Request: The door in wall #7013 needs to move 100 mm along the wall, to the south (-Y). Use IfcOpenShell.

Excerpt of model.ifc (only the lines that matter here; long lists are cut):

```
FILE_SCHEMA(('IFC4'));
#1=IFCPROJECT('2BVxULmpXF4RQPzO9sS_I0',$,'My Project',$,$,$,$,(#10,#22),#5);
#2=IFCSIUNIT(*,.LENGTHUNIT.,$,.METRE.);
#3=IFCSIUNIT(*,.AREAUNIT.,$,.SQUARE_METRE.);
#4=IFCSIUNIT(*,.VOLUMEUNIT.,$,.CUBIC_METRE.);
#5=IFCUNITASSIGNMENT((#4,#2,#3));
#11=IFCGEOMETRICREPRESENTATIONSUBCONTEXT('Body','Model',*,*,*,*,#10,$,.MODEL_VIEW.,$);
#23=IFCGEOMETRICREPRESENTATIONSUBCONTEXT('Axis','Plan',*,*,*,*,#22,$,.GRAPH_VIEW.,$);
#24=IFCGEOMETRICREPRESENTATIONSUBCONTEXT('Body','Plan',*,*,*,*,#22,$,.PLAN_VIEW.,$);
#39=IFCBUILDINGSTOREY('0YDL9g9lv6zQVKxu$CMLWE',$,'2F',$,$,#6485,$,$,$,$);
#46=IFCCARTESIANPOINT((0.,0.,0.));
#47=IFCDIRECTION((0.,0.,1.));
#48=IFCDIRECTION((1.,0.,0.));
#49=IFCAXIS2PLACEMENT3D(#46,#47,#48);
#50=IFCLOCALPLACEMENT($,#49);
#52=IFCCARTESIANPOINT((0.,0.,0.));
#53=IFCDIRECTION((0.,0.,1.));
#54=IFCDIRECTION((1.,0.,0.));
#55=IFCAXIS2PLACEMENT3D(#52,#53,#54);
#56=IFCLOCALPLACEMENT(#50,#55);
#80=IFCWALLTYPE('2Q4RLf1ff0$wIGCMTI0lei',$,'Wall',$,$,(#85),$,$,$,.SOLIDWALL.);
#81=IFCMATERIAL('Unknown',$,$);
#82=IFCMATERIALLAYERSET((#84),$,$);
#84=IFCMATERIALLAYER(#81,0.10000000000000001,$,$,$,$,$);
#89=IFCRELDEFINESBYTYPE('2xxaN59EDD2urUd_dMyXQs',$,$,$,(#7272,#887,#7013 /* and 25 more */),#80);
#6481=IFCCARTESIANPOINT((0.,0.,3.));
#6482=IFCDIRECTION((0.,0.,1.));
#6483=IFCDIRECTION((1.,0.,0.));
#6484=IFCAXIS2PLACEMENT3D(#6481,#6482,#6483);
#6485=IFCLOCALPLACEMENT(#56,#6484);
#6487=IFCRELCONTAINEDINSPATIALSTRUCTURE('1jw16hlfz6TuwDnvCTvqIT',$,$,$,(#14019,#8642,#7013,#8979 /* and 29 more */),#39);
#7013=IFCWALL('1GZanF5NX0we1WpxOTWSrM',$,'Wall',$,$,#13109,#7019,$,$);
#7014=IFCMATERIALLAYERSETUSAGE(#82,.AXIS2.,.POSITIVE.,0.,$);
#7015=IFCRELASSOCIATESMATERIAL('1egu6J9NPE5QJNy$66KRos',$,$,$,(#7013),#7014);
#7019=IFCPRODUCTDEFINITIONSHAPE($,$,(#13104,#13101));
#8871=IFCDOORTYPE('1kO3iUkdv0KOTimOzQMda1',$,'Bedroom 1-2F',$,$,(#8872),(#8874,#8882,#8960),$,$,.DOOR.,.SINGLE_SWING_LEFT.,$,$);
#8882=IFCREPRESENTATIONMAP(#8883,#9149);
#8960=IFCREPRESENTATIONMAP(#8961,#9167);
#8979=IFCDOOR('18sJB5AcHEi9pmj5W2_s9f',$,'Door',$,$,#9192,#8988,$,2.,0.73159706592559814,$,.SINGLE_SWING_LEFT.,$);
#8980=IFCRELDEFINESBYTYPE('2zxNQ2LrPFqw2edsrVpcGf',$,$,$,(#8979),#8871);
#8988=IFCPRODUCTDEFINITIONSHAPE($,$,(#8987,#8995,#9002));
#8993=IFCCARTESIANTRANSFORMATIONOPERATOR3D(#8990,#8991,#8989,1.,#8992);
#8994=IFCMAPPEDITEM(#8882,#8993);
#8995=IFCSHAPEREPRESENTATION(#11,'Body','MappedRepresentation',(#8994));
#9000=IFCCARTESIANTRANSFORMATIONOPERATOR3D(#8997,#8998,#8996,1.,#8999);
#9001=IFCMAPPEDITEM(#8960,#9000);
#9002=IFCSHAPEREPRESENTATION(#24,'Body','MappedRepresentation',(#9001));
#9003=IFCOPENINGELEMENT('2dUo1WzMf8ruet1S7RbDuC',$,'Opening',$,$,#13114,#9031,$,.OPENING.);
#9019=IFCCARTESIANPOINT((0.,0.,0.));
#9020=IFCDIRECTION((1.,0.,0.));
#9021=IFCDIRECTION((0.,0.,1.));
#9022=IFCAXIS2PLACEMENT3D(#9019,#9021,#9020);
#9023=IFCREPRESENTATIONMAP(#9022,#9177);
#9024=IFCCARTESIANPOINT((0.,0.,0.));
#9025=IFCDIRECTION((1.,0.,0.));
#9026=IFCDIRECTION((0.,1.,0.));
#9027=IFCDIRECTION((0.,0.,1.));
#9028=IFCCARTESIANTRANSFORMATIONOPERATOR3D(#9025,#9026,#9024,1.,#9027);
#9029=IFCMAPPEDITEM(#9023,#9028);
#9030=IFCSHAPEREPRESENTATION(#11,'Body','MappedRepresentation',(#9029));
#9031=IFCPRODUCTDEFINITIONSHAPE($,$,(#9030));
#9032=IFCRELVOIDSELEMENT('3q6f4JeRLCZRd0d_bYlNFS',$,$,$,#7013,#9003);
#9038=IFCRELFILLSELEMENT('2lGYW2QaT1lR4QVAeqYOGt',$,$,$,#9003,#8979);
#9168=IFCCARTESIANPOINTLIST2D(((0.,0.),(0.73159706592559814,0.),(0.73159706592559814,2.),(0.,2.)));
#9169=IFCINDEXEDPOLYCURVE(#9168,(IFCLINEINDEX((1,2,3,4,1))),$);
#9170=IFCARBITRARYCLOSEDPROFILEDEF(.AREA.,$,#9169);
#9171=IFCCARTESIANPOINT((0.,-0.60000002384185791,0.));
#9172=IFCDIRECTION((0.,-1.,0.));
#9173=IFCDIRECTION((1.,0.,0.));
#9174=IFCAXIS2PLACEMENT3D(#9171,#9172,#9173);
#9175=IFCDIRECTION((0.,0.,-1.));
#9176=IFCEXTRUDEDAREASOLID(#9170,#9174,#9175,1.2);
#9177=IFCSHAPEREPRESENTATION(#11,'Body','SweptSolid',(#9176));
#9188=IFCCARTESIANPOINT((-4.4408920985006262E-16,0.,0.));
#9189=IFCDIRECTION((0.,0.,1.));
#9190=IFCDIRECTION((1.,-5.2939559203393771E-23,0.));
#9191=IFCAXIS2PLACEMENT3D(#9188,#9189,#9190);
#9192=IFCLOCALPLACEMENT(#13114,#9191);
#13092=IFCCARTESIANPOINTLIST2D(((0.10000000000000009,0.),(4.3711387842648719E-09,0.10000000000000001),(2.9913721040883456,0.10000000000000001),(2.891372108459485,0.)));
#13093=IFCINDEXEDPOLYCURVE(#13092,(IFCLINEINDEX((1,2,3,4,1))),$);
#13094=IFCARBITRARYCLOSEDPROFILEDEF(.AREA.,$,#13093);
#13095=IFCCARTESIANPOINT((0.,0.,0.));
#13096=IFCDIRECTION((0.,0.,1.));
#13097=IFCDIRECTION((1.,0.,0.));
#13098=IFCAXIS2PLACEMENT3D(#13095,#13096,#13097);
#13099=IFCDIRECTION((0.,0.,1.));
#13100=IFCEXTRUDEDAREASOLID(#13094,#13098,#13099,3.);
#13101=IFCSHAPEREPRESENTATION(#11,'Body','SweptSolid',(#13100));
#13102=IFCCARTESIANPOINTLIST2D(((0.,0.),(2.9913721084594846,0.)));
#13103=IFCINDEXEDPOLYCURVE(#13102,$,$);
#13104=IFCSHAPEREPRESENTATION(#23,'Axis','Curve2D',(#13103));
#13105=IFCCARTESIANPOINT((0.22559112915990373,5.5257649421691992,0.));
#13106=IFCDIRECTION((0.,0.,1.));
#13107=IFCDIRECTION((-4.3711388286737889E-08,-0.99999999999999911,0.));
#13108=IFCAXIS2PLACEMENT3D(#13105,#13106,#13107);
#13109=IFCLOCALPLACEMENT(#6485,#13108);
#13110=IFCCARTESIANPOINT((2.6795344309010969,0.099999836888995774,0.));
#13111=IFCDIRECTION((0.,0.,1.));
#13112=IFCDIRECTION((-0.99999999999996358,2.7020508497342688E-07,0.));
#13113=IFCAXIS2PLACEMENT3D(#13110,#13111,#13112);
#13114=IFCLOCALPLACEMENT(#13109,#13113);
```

```python
import ifcopenshell
import ifcopenshell.api.geometry
import ifcopenshell.util.placement
import ifcopenshell.util.unit

model = ifcopenshell.open("model.ifc")
unit_scale = ifcopenshell.util.unit.calculate_unit_scale(model)

door = model.by_guid("18sJB5AcHEi9pmj5W2_s9f")
opening = door.FillsVoids[0].RelatingOpeningElement
wall = opening.VoidsElements[0].RelatingBuildingElement

wall_matrix = ifcopenshell.util.placement.get_local_placement(wall.ObjectPlacement)
shift = wall_matrix[:3, 0] * 0.1 / unit_scale
before = ifcopenshell.util.placement.get_local_placement(door.ObjectPlacement)[:3, 3].copy()

# The door is placed relative to its opening, so it follows when the opening moves.
matrix = ifcopenshell.util.placement.get_local_placement(opening.ObjectPlacement)
matrix[:3, 3] += shift
ifcopenshell.api.geometry.edit_object_placement(
    model, product=opening, matrix=matrix, is_si=False, should_transform_children=True
)

after = ifcopenshell.util.placement.get_local_placement(door.ObjectPlacement)[:3, 3]
print("door moved by", (after - before).round(3) + 0.0)

model.write("model_edited.ifc")
```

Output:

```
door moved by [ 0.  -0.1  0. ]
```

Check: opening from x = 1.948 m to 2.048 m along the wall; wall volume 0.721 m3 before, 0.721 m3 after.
